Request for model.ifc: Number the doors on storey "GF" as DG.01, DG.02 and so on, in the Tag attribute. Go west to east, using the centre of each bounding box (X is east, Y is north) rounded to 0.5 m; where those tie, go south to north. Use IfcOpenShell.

First a look at what the model holds.

```python
import ifcopenshell
import ifcopenshell.util.element
import ifcopenshell.util.placement

model = ifcopenshell.open("model.ifc")
print(model.schema)
storey = next(s for s in model.by_type("IfcBuildingStorey") if s.Name == "GF")
doors = [e for e in ifcopenshell.util.element.get_decomposition(storey) if e.is_a("IfcDoor")]
for e in sorted(doors, key=lambda e: e.id()):
    origin = ifcopenshell.util.placement.get_local_placement(e.ObjectPlacement)[:3, 3]
    print(e.id(), e.Tag, e.Name, origin.round(2) + 0.0, sep=" | ")
```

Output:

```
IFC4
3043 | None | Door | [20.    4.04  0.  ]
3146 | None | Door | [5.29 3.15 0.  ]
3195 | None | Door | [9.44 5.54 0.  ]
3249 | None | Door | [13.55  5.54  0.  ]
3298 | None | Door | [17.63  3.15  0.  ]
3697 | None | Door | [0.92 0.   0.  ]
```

```python
import ifcopenshell
import ifcopenshell.geom
import ifcopenshell.util.element
import ifcopenshell.util.shape

model = ifcopenshell.open("model.ifc")
settings = ifcopenshell.geom.settings()
settings.set("use-world-coords", True)


def centre(element):
    shape = ifcopenshell.geom.create_shape(settings, element)
    return ifcopenshell.util.shape.get_bbox_centroid(shape.geometry)


storey = next(s for s in model.by_type("IfcBuildingStorey") if s.Name == "GF")
doors = [e for e in ifcopenshell.util.element.get_decomposition(storey) if e.is_a("IfcDoor")]

# Insertion points can sit at a corner or the storey origin, so sort by the geometry (in metres).
centres = {e: centre(e) for e in doors}
doors.sort(key=lambda e: (round(centres[e][0] / 0.5), centres[e][1]))

for i, e in enumerate(doors, start=1):
    number = f"DG.{i:02d}"
    e.Tag = number
    print(e.id(), number)

model.write("model_rev.ifc")
```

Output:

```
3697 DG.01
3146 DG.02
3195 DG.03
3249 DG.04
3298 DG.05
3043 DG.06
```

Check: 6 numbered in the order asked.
